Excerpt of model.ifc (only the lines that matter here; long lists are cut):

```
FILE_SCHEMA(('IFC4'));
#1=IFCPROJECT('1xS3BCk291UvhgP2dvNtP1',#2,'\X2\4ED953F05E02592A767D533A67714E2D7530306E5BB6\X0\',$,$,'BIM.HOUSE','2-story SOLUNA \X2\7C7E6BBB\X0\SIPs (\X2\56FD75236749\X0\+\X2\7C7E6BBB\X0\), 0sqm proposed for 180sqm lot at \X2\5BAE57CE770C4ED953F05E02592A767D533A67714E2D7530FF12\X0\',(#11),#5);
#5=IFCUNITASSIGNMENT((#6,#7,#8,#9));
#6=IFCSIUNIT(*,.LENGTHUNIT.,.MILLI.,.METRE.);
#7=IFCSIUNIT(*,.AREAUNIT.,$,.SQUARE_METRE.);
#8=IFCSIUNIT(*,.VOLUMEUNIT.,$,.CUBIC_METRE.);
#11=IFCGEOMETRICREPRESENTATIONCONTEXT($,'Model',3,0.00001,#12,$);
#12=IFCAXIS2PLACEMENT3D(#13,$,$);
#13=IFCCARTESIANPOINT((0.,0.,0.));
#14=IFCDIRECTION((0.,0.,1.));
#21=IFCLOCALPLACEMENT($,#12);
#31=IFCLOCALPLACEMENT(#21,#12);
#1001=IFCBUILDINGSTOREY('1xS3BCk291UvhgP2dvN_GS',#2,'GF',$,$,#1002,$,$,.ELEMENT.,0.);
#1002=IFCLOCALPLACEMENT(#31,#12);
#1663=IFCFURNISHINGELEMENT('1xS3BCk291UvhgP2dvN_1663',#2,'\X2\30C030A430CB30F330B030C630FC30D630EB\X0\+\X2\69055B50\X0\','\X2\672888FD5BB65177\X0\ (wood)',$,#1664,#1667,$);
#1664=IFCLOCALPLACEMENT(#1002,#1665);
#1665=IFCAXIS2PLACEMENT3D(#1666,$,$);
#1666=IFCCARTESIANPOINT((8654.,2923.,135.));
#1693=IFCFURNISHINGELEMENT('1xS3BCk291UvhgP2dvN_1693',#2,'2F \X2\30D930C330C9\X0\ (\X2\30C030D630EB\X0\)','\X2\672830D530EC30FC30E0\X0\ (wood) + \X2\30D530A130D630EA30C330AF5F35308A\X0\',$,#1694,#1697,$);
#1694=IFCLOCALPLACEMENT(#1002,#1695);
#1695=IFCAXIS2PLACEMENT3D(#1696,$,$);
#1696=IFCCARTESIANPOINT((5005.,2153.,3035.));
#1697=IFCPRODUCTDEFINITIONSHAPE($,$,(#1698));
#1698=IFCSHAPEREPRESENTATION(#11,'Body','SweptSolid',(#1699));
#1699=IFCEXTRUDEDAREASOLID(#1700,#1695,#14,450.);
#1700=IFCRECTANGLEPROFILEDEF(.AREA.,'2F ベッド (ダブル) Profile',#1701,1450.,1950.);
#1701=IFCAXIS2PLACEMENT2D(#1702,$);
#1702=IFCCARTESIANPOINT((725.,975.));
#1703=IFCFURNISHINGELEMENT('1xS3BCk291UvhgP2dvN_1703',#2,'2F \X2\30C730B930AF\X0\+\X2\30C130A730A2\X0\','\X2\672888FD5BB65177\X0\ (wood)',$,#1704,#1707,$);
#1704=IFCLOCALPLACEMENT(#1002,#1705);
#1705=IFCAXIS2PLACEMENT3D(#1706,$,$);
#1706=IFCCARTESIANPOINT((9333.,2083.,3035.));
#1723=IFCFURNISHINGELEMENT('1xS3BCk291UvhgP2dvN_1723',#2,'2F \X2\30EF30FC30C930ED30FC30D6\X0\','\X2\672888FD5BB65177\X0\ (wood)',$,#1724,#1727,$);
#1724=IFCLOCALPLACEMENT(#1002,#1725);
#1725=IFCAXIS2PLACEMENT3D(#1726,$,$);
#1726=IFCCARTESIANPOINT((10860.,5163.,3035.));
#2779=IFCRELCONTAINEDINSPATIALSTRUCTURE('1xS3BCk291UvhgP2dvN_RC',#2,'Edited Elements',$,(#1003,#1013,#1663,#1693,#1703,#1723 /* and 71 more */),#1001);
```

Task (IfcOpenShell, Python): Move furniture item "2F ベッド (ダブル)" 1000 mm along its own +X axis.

```python
import ifcopenshell
import ifcopenshell.api.geometry
import ifcopenshell.util.placement
import ifcopenshell.util.unit

model = ifcopenshell.open("model.ifc")
unit_scale = ifcopenshell.util.unit.calculate_unit_scale(model)

item = model.by_guid("1xS3BCk291UvhgP2dvN_1693")
matrix = ifcopenshell.util.placement.get_local_placement(item.ObjectPlacement)
matrix[:3, 3] += matrix[:3, 0] * 1 / unit_scale
ifcopenshell.api.geometry.edit_object_placement(model, product=item, matrix=matrix, is_si=False)

print(ifcopenshell.util.placement.get_local_placement(item.ObjectPlacement).round(3) + 0.0)

model.write("model-out.ifc")
```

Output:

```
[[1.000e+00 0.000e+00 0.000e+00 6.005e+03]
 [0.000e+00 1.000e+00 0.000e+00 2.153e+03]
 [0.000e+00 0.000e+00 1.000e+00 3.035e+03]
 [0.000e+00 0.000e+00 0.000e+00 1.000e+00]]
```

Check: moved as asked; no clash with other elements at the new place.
